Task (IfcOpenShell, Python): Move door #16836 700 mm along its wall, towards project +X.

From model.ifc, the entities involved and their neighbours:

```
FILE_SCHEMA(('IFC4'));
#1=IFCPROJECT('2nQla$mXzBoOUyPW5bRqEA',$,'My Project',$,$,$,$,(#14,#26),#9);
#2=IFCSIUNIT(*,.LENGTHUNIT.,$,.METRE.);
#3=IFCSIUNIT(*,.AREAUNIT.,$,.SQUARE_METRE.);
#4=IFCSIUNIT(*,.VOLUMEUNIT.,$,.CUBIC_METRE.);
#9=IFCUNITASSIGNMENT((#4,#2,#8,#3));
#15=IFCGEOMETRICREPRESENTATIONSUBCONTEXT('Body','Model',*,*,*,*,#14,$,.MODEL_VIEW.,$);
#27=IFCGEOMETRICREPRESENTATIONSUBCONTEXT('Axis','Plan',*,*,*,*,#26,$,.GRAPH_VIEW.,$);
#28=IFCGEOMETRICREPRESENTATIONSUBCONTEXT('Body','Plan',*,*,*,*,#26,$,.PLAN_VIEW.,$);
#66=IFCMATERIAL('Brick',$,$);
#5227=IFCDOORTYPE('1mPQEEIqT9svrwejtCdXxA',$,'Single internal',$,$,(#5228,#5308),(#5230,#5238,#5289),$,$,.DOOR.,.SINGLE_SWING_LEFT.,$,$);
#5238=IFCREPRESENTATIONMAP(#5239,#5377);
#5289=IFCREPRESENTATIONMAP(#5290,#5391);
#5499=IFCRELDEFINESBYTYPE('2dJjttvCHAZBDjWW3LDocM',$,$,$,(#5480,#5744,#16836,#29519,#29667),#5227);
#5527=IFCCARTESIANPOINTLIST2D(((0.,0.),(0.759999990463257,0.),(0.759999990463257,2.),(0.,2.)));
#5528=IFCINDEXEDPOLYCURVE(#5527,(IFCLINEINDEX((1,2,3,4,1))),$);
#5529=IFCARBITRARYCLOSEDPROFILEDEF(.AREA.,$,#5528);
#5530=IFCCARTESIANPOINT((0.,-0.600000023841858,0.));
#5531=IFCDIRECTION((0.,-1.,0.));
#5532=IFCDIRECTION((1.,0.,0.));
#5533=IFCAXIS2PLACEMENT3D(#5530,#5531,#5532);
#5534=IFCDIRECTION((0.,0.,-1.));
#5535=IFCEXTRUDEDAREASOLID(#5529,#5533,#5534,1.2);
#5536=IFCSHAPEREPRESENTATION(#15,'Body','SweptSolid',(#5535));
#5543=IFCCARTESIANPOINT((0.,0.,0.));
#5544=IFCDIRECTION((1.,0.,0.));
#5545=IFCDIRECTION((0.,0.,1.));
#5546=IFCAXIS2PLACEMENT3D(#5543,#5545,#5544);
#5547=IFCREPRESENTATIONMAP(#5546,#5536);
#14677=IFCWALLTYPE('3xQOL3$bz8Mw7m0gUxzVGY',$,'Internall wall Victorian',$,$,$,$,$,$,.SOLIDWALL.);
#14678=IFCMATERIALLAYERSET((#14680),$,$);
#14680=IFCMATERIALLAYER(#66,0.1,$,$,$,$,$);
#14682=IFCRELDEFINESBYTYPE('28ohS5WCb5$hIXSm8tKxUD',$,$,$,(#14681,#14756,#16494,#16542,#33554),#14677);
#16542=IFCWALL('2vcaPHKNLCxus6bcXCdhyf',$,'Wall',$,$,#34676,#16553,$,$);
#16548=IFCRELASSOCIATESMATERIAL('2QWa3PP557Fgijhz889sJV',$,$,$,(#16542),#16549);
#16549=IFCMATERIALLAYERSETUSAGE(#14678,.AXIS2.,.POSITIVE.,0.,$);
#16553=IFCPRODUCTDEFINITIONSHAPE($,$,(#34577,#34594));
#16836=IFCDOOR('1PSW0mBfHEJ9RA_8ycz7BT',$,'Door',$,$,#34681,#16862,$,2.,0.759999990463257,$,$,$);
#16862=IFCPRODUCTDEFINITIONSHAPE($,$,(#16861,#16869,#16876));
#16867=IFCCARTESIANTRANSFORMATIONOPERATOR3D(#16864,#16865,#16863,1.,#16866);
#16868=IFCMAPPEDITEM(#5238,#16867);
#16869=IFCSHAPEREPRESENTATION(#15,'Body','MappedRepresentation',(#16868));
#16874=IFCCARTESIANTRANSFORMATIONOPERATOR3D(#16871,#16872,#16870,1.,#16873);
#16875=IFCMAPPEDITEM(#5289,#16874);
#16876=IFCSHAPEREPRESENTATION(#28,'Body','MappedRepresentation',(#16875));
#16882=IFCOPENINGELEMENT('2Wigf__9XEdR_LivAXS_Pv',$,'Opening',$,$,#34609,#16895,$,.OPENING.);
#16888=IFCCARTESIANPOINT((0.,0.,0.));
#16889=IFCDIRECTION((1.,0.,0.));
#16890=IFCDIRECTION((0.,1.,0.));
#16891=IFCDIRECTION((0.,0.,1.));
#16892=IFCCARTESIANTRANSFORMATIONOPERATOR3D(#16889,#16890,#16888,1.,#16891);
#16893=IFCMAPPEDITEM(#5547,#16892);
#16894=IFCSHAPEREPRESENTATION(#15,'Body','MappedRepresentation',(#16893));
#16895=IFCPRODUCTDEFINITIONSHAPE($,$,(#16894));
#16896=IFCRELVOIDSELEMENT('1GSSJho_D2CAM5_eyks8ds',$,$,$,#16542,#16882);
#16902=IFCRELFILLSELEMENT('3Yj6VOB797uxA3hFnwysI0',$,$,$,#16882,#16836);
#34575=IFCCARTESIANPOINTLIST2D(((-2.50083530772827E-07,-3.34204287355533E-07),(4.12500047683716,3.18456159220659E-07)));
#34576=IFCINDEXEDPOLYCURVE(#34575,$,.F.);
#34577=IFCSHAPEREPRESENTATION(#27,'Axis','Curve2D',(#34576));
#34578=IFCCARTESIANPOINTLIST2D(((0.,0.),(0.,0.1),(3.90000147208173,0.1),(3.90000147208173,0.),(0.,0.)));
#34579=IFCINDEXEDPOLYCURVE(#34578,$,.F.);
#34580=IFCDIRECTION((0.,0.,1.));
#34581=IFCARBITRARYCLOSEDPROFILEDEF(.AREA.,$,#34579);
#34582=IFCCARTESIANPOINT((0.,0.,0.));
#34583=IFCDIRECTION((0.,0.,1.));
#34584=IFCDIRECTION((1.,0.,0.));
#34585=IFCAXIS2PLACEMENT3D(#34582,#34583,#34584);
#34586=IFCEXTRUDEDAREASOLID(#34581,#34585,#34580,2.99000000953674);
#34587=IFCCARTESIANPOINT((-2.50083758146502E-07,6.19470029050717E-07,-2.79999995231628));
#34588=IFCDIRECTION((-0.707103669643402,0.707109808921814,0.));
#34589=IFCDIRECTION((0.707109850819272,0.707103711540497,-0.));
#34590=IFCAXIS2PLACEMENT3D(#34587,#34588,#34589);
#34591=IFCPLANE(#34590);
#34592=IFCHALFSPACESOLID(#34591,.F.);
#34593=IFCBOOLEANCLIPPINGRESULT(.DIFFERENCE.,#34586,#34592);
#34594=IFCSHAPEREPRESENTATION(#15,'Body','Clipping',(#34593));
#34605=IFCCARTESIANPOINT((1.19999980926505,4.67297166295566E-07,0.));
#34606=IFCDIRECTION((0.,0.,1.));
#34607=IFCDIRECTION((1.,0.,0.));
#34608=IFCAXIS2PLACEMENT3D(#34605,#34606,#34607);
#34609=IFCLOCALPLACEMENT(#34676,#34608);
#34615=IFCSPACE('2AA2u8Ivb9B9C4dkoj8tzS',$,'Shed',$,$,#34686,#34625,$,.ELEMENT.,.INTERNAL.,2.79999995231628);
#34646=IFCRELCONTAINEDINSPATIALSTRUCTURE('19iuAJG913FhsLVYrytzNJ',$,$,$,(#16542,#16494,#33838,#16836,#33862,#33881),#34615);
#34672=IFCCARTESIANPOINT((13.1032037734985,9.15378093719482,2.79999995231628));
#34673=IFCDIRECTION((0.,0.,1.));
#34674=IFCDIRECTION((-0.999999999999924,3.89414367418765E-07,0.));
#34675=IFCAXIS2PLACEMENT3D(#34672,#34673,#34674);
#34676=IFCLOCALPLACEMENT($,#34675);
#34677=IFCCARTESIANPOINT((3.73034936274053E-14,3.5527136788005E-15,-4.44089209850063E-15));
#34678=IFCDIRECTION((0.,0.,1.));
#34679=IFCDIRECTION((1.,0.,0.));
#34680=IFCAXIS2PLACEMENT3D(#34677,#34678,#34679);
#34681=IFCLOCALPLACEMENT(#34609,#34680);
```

```python
import ifcopenshell
import ifcopenshell.api.geometry
import ifcopenshell.util.placement
import ifcopenshell.util.unit

model = ifcopenshell.open("model.ifc")
unit_scale = ifcopenshell.util.unit.calculate_unit_scale(model)

door = model.by_guid("1PSW0mBfHEJ9RA_8ycz7BT")
opening = door.FillsVoids[0].RelatingOpeningElement
wall = opening.VoidsElements[0].RelatingBuildingElement

wall_matrix = ifcopenshell.util.placement.get_local_placement(wall.ObjectPlacement)
shift = wall_matrix[:3, 0] * -0.7 / unit_scale
before = ifcopenshell.util.placement.get_local_placement(door.ObjectPlacement)[:3, 3].copy()

# The door is placed relative to its opening, so it follows when the opening moves.
matrix = ifcopenshell.util.placement.get_local_placement(opening.ObjectPlacement)
matrix[:3, 3] += shift
ifcopenshell.api.geometry.edit_object_placement(
    model, product=opening, matrix=matrix, is_si=False, should_transform_children=True
)

after = ifcopenshell.util.placement.get_local_placement(door.ObjectPlacement)[:3, 3]
print("door moved by", (after - before).round(3) + 0.0)

model.write("model_updated.ifc")
```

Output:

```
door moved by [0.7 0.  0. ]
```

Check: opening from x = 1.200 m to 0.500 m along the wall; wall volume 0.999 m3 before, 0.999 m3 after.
